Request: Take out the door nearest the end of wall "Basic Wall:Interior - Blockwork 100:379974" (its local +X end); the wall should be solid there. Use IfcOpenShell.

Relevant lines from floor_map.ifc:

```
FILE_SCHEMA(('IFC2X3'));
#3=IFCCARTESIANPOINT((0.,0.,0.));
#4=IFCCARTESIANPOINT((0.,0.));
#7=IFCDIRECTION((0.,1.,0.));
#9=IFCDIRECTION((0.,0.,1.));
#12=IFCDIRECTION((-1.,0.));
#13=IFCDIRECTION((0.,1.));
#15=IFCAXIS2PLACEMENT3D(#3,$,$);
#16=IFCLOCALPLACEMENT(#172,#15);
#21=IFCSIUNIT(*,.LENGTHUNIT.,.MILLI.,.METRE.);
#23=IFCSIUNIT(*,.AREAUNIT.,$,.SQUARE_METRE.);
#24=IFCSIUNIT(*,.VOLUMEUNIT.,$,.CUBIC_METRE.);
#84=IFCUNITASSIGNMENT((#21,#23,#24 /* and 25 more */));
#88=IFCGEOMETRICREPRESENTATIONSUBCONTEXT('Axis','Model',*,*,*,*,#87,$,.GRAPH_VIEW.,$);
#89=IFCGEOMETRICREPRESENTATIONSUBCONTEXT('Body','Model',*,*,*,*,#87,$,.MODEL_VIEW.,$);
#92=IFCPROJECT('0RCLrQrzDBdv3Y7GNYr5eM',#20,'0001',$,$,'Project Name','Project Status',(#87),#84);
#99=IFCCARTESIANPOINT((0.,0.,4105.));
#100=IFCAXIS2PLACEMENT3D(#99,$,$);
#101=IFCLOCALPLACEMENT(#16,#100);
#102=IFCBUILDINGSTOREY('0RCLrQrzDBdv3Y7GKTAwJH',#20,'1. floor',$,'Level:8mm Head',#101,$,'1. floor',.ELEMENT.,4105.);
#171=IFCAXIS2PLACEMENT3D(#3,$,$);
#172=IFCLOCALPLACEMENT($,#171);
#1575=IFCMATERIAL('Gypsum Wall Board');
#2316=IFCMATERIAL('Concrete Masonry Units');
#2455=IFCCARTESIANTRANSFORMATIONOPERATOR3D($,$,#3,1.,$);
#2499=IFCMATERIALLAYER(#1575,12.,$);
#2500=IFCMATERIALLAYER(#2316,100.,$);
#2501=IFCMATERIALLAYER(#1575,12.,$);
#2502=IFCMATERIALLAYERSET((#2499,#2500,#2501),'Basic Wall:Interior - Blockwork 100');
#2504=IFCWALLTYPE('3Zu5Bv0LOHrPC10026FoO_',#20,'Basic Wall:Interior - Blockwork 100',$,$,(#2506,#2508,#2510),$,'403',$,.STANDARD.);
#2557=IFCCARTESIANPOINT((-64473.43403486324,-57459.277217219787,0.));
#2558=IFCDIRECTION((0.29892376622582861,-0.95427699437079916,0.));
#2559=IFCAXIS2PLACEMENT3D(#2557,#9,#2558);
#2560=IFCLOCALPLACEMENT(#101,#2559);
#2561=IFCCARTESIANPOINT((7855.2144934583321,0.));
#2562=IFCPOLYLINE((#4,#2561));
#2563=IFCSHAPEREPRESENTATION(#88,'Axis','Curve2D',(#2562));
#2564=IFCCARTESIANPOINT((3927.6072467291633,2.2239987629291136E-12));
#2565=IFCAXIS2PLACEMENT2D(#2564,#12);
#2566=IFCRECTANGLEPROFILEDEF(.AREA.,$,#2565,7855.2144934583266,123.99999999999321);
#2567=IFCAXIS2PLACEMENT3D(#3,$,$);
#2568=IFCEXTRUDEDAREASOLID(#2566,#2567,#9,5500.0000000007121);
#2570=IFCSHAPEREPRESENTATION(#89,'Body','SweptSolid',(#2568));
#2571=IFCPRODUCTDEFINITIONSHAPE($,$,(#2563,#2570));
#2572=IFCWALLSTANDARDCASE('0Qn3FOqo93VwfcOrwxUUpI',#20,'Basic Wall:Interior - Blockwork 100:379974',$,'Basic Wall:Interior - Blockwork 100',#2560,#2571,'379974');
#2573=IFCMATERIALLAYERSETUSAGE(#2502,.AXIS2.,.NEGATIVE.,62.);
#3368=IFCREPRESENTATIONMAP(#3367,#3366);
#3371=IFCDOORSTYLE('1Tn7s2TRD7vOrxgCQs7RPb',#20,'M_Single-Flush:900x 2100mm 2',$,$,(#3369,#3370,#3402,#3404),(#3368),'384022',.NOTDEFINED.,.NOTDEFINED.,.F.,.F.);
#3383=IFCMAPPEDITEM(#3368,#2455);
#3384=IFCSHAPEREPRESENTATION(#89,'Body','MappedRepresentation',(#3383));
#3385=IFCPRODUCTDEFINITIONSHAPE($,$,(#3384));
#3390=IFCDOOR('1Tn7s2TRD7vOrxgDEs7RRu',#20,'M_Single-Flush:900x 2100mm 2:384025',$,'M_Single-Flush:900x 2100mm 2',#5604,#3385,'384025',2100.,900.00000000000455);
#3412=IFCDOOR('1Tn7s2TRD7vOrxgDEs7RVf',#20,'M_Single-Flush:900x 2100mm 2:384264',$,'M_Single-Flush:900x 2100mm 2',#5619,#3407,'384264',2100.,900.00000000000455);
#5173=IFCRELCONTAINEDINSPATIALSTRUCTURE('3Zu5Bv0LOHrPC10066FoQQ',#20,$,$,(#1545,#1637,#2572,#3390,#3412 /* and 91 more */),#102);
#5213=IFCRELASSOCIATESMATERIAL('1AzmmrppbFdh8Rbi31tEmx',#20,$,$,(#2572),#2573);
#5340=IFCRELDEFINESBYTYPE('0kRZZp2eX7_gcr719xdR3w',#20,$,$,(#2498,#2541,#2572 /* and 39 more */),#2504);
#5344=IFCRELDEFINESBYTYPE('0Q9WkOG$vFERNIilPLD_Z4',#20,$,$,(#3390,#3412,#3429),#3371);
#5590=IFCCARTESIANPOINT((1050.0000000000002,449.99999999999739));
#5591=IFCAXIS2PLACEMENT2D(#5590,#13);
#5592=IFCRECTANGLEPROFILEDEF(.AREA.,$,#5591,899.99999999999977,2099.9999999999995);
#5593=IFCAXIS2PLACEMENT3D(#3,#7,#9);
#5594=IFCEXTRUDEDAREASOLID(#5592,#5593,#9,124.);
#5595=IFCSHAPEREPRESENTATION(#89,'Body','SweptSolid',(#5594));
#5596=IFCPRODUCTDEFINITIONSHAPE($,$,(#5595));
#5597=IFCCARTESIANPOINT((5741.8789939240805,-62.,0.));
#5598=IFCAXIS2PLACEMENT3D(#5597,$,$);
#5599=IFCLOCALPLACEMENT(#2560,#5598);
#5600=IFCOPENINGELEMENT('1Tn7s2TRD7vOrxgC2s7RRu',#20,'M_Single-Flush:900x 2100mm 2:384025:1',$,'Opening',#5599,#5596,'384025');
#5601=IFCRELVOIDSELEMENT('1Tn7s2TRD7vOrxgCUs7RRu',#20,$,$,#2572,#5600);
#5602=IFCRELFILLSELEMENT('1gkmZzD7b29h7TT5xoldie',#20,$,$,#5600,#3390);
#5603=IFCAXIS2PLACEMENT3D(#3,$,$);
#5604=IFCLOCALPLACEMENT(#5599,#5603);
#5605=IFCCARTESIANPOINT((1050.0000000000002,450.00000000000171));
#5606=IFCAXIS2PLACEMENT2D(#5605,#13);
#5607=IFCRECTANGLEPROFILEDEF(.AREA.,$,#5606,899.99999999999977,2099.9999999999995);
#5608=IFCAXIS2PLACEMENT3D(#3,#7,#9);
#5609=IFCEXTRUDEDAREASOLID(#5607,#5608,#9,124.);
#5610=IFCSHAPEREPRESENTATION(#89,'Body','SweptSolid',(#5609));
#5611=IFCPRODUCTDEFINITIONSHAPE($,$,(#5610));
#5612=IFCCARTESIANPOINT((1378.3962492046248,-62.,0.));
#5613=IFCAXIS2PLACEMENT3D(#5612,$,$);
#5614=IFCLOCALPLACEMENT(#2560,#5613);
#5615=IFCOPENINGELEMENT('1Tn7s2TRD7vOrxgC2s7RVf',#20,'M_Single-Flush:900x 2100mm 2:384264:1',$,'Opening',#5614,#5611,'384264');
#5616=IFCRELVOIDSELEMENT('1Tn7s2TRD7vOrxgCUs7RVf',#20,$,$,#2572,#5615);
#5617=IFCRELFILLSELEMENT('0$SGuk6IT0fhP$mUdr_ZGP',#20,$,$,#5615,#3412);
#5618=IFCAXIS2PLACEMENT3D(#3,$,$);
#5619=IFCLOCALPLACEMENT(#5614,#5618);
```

```python
import ifcopenshell
import ifcopenshell.api.feature
import ifcopenshell.api.root
import ifcopenshell.geom
import ifcopenshell.util.shape

model = ifcopenshell.open("floor_map.ifc")
settings = ifcopenshell.geom.settings()


def volume(element):
    """Net volume in cubic metres, openings subtracted."""
    shape = ifcopenshell.geom.create_shape(settings, element)
    return ifcopenshell.util.shape.get_volume(shape.geometry)


door = model.by_id(3390)
opening = door.FillsVoids[0].RelatingOpeningElement
wall = opening.VoidsElements[0].RelatingBuildingElement
before = volume(wall)

ifcopenshell.api.root.remove_product(model, product=door)
ifcopenshell.api.feature.remove_feature(model, feature=opening)

after = volume(wall)

print(f"wall volume {before:.3f} -> {after:.3f} m3")

model.write("floor_map_rev.ifc")
```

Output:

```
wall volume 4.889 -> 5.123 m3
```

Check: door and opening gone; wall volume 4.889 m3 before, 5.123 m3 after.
